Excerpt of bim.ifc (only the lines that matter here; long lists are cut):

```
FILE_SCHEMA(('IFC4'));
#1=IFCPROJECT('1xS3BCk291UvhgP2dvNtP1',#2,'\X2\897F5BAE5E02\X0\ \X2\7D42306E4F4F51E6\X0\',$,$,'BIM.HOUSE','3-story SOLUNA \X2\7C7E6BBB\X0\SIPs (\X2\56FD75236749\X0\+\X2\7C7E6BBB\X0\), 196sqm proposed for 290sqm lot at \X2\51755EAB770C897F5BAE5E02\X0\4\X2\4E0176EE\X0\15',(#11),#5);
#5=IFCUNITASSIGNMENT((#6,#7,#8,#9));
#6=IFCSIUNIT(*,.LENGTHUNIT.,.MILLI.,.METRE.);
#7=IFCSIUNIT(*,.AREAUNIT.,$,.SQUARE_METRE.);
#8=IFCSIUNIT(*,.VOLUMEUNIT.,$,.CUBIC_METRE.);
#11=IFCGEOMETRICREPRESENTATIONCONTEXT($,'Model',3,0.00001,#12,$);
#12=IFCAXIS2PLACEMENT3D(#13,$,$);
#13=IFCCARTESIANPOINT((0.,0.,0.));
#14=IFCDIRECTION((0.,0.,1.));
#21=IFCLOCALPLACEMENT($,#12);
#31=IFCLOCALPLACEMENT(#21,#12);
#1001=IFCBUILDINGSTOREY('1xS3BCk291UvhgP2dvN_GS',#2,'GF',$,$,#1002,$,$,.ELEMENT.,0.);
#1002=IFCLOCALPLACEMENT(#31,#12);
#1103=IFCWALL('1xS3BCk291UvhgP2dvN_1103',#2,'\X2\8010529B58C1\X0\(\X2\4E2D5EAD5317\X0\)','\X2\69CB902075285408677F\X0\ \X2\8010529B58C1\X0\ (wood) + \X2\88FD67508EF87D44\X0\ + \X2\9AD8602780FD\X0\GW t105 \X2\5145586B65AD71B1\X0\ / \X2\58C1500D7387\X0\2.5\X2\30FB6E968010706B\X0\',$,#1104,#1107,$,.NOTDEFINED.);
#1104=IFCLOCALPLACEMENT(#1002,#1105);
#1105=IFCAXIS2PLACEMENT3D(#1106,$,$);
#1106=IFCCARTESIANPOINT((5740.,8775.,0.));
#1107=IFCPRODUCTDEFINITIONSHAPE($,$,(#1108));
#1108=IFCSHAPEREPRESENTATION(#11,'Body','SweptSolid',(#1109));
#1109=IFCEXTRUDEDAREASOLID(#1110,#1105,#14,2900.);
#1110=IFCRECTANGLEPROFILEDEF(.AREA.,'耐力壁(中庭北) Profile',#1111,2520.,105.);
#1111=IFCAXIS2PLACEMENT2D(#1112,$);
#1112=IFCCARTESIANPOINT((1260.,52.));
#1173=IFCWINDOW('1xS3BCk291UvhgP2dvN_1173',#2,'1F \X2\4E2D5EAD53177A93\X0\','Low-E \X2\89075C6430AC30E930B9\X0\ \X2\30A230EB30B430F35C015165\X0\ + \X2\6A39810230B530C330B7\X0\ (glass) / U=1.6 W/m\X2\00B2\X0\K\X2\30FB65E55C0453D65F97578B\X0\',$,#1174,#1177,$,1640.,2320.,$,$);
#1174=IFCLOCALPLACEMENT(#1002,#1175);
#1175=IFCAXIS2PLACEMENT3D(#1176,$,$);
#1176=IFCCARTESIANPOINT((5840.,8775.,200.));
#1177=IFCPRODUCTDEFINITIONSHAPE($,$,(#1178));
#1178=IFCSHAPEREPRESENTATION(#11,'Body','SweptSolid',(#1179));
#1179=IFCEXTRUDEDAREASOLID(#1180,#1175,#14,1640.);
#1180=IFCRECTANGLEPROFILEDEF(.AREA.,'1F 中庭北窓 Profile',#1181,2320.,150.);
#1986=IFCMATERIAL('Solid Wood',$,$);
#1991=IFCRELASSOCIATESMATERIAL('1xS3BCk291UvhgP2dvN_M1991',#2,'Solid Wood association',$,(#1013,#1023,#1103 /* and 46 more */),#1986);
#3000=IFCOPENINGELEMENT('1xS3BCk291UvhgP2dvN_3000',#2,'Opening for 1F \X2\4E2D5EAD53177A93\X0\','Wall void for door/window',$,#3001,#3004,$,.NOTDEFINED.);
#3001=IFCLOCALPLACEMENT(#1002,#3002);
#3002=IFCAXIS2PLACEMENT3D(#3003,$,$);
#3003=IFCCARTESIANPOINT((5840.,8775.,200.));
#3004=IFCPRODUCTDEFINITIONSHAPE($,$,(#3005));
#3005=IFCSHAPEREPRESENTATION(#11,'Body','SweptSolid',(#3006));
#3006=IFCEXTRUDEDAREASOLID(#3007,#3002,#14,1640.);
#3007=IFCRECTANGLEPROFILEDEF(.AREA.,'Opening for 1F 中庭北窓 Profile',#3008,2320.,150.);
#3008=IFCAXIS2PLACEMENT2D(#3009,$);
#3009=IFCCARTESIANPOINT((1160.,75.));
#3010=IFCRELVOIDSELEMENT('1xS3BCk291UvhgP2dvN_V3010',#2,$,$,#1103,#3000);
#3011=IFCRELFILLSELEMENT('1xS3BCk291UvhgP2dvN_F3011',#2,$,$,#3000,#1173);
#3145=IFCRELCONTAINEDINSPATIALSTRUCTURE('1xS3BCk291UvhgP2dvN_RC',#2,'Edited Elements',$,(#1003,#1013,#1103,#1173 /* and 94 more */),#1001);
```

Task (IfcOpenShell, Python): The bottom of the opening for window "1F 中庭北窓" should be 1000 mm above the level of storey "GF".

```python
import numpy as np
import ifcopenshell
import ifcopenshell.api.geometry
import ifcopenshell.geom
import ifcopenshell.util.element
import ifcopenshell.util.placement
import ifcopenshell.util.shape
import ifcopenshell.util.unit

model = ifcopenshell.open("bim.ifc")
unit_scale = ifcopenshell.util.unit.calculate_unit_scale(model)

window = model.by_guid("1xS3BCk291UvhgP2dvN_1173")
opening = window.FillsVoids[0].RelatingOpeningElement
storey = ifcopenshell.util.element.get_container(window, ifc_class="IfcBuildingStorey")
level = ifcopenshell.util.placement.get_local_placement(storey.ObjectPlacement)[2, 3]

# The opening's origin need not be at the sill, so measure its lowest point.
shape = ifcopenshell.geom.create_shape(ifcopenshell.geom.settings(), opening)
bottom = ifcopenshell.util.shape.get_shape_bottom_elevation(shape, shape.geometry) / unit_scale
dz = level + 1000.0 - bottom

shift = np.array([0.0, 0.0, dz])
# The window is not placed relative to its opening, so move both.
for product in (opening, window):
    matrix = ifcopenshell.util.placement.get_local_placement(product.ObjectPlacement)
    matrix[:3, 3] += shift
    ifcopenshell.api.geometry.edit_object_placement(model, product=product, matrix=matrix, is_si=False)

print(f"moved by {dz * unit_scale:+.3f} m")

model.write("bim_rev.ifc")
```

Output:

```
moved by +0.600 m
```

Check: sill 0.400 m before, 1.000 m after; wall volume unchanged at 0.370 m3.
